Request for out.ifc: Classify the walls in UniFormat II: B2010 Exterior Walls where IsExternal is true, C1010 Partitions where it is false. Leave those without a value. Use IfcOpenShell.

First a look at what the model holds.

```python
import ifcopenshell
import ifcopenshell.util.element

model = ifcopenshell.open("out.ifc")
print(model.schema)
print("classifications:", [c.Name for c in model.by_type("IfcClassification")])
values = [ifcopenshell.util.element.get_pset(e, "Pset_WallCommon", "IsExternal") for e in model.by_type("IfcWall")]
for value in (True, False, None):
    print("IsExternal", value, values.count(value))
```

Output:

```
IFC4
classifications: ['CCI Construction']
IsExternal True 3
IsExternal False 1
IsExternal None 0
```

```python
import ifcopenshell
import ifcopenshell.api.classification
import ifcopenshell.util.element

model = ifcopenshell.open("out.ifc")

system = ifcopenshell.api.classification.add_classification(model, classification="UniFormat II")

walls = model.by_type("IfcWall")
external = {e: ifcopenshell.util.element.get_pset(e, "Pset_WallCommon", "IsExternal") for e in walls}
for flag, code, name in ((True, "B2010", "Exterior Walls"), (False, "C1010", "Partitions")):
    products = [e for e in walls if external[e] is flag]
    ifcopenshell.api.classification.add_reference(
        model, products=products, classification=system, identification=code, name=name
    )
    print(code, len(products))

model.write("out_v2.ifc")
```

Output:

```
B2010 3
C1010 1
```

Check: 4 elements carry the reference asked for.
